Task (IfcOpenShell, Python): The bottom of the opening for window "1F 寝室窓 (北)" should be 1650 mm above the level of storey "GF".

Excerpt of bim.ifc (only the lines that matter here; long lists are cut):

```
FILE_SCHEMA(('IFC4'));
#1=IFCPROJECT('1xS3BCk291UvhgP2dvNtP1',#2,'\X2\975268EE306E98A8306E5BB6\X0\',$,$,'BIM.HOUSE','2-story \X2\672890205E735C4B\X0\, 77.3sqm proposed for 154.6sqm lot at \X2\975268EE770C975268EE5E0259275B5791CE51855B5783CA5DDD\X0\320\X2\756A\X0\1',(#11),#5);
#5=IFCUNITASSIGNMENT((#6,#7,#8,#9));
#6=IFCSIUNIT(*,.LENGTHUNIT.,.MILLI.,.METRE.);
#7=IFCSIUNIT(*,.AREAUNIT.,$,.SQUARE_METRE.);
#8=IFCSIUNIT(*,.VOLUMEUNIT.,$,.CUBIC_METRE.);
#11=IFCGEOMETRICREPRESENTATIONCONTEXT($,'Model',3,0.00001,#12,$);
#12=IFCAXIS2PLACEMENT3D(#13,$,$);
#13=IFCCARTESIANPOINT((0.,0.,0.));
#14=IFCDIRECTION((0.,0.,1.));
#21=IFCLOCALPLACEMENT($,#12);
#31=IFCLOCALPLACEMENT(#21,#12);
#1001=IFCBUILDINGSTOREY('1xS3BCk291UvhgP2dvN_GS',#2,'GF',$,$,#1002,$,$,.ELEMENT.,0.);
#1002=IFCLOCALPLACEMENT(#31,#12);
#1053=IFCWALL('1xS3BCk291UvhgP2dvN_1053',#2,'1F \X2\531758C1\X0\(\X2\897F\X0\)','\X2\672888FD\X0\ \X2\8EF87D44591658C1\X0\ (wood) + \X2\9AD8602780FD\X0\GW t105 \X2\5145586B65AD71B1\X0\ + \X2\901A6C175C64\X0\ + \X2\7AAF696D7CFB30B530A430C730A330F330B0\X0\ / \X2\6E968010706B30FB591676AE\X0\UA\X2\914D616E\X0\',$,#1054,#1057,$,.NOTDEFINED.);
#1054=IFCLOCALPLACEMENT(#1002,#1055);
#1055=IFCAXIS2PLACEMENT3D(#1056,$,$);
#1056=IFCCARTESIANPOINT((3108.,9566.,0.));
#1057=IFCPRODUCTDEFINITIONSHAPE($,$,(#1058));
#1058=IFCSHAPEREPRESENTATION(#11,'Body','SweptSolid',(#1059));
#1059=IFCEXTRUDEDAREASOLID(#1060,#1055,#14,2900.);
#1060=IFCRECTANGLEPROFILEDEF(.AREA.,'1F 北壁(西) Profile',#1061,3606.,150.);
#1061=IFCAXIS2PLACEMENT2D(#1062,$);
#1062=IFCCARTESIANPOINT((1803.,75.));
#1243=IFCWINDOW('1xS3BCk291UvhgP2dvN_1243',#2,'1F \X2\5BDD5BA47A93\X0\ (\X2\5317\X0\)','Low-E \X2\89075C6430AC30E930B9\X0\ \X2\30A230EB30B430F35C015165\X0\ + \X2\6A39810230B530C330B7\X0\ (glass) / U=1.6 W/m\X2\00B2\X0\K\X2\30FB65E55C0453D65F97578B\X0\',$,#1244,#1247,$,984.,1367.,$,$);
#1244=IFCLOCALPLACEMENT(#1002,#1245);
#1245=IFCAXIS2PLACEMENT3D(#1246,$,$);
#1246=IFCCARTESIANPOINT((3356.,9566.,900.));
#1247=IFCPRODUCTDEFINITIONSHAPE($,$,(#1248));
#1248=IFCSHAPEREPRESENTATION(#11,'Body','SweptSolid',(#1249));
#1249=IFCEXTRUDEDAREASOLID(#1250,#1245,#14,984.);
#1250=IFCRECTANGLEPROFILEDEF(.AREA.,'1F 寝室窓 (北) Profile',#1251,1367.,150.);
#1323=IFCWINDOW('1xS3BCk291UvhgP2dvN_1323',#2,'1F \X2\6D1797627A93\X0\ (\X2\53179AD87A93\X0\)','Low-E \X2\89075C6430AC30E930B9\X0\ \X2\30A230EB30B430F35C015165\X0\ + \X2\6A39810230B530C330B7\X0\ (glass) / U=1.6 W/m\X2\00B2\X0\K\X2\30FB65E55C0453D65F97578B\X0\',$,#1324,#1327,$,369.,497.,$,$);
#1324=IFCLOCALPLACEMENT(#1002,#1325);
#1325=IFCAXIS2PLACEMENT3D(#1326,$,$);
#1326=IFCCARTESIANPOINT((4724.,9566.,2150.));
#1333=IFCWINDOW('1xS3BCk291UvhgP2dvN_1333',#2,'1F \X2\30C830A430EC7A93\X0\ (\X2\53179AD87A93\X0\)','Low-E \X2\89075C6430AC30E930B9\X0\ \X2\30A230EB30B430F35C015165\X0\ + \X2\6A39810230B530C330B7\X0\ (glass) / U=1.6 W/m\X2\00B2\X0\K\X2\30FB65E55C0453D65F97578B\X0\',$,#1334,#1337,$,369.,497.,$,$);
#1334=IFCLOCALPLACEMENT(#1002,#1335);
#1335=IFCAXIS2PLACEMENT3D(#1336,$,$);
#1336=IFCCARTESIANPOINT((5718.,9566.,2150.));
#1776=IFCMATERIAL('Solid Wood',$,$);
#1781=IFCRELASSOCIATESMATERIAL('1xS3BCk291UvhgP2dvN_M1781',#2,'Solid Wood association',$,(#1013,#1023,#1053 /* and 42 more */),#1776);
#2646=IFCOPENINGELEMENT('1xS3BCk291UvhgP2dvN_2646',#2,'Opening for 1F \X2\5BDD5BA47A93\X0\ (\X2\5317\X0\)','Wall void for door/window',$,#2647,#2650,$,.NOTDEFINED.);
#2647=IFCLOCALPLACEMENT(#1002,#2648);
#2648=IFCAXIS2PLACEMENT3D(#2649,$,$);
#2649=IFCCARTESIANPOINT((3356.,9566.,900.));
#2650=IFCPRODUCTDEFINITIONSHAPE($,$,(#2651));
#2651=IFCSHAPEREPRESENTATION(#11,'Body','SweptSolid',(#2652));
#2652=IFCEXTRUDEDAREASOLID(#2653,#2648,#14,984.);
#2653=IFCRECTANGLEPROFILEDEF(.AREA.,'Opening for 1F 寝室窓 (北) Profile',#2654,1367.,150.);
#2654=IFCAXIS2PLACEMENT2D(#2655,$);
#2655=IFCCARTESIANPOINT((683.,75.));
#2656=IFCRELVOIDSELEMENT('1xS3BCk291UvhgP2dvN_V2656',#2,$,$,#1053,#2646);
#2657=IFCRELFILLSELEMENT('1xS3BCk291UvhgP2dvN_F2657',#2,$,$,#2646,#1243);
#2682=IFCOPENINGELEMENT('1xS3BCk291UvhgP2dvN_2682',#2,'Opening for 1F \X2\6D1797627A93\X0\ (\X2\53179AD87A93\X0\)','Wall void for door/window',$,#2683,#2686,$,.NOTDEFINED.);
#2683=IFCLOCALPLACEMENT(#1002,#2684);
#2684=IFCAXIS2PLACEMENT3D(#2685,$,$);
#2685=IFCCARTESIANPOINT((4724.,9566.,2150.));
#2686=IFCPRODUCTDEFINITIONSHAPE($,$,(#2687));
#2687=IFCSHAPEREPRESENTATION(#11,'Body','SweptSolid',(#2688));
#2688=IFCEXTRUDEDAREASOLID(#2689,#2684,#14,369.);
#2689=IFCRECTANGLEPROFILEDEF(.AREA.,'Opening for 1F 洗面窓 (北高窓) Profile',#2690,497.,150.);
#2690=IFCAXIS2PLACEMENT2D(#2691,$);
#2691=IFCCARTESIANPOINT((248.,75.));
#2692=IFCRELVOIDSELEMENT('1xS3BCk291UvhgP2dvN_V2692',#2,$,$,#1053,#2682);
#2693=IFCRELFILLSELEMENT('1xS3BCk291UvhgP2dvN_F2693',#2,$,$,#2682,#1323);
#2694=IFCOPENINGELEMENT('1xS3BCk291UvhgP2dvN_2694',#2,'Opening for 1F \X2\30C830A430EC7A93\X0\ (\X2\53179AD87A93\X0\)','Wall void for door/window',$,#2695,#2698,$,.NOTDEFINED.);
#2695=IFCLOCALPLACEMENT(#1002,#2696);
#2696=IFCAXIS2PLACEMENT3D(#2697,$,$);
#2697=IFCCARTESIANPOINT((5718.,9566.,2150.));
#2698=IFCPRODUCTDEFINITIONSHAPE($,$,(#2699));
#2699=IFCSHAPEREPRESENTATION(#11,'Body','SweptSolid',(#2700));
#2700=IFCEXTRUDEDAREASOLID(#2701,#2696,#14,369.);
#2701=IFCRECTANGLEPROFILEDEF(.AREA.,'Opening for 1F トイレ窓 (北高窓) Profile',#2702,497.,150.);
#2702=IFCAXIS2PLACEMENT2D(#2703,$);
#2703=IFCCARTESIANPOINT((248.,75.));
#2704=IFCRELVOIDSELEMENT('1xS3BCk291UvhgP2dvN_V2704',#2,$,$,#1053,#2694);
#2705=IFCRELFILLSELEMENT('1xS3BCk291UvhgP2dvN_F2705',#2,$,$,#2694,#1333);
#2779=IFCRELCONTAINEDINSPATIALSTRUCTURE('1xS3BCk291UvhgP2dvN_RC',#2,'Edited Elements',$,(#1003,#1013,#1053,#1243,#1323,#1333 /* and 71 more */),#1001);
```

```python
import numpy as np
import ifcopenshell
import ifcopenshell.api.geometry
import ifcopenshell.geom
import ifcopenshell.util.element
import ifcopenshell.util.placement
import ifcopenshell.util.shape
import ifcopenshell.util.unit

model = ifcopenshell.open("bim.ifc")
unit_scale = ifcopenshell.util.unit.calculate_unit_scale(model)

window = model.by_guid("1xS3BCk291UvhgP2dvN_1243")
opening = window.FillsVoids[0].RelatingOpeningElement
storey = ifcopenshell.util.element.get_container(window, ifc_class="IfcBuildingStorey")
level = ifcopenshell.util.placement.get_local_placement(storey.ObjectPlacement)[2, 3]

# The opening's origin need not be at the sill, so measure its lowest point.
shape = ifcopenshell.geom.create_shape(ifcopenshell.geom.settings(), opening)
bottom = ifcopenshell.util.shape.get_shape_bottom_elevation(shape, shape.geometry) / unit_scale
dz = level + 1.65 / unit_scale - bottom

shift = np.array([0.0, 0.0, dz])
# The window is not placed relative to its opening, so move both.
for product in (opening, window):
    matrix = ifcopenshell.util.placement.get_local_placement(product.ObjectPlacement)
    matrix[:3, 3] += shift
    ifcopenshell.api.geometry.edit_object_placement(model, product=product, matrix=matrix, is_si=False)

print(f"moved by {dz * unit_scale:+.3f} m")

model.write("bim-out.ifc")
```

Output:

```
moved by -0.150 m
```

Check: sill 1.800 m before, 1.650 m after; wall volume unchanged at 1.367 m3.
